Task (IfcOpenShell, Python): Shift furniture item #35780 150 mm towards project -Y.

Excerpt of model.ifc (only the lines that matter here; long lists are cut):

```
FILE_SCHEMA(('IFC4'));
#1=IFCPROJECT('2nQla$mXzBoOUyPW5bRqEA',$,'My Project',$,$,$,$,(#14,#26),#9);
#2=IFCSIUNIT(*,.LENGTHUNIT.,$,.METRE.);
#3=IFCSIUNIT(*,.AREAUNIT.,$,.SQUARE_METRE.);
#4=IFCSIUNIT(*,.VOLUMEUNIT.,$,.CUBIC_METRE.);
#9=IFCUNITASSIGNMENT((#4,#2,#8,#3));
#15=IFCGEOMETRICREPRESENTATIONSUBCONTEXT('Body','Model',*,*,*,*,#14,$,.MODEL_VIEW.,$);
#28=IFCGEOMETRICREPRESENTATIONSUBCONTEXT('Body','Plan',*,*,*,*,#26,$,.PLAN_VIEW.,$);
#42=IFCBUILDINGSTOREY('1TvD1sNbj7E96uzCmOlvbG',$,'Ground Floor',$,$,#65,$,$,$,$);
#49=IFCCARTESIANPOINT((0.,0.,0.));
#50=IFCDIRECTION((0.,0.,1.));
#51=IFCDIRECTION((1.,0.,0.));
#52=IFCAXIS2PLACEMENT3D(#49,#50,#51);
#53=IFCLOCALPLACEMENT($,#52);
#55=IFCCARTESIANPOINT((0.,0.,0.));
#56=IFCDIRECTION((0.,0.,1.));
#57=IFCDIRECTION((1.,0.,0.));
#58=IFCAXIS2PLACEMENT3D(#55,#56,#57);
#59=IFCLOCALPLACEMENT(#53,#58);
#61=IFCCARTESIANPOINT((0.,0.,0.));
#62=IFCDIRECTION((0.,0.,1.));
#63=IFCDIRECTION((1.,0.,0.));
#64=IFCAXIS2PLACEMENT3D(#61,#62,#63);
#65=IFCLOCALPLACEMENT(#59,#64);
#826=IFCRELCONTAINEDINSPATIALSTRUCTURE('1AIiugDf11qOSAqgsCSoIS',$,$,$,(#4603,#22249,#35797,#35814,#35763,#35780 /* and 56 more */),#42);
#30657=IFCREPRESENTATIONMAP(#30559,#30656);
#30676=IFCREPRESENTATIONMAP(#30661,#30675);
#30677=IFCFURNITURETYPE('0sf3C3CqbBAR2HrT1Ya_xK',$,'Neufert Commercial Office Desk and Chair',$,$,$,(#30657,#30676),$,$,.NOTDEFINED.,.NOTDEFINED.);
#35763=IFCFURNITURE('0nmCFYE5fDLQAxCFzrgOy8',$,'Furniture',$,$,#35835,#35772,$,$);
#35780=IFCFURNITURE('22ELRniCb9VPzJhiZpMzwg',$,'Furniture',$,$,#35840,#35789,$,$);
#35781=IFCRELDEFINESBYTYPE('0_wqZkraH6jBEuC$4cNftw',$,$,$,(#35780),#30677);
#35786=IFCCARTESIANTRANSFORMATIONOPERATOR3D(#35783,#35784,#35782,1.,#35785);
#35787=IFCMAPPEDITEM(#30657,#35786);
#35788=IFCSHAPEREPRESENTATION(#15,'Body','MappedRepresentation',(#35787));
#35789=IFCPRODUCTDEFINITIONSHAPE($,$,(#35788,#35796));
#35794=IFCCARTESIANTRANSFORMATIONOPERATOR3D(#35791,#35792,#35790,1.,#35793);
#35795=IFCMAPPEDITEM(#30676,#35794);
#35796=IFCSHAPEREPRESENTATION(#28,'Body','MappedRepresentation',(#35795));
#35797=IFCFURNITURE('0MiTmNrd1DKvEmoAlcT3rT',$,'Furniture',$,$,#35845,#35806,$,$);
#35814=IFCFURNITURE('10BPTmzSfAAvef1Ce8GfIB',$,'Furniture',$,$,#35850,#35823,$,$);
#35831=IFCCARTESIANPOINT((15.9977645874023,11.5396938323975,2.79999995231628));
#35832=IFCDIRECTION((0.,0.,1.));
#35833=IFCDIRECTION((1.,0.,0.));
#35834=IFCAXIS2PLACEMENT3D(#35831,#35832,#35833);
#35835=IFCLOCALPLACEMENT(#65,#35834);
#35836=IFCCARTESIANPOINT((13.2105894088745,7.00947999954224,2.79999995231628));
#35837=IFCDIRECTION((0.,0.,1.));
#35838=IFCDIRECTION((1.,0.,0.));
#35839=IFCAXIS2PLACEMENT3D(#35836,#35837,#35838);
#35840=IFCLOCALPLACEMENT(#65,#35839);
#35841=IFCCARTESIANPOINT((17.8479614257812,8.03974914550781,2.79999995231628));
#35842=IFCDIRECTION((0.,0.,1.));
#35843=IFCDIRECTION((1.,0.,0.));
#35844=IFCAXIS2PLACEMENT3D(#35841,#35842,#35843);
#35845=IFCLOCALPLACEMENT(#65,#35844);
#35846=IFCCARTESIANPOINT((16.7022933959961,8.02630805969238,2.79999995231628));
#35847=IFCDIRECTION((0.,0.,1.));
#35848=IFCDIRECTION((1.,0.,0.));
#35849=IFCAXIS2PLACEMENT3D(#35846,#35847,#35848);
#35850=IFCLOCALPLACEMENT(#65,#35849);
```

```python
import ifcopenshell
import ifcopenshell.api.geometry
import ifcopenshell.util.placement
import ifcopenshell.util.unit

model = ifcopenshell.open("model.ifc")
unit_scale = ifcopenshell.util.unit.calculate_unit_scale(model)

item = model.by_id(35780)
matrix = ifcopenshell.util.placement.get_local_placement(item.ObjectPlacement)
matrix[1, 3] -= 0.15 / unit_scale
ifcopenshell.api.geometry.edit_object_placement(model, product=item, matrix=matrix, is_si=False)

print(ifcopenshell.util.placement.get_local_placement(item.ObjectPlacement).round(3) + 0.0)

model.write("model_v2.ifc")
```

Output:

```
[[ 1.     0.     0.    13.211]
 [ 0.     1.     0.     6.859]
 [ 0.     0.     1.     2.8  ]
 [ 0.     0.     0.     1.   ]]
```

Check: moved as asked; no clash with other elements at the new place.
